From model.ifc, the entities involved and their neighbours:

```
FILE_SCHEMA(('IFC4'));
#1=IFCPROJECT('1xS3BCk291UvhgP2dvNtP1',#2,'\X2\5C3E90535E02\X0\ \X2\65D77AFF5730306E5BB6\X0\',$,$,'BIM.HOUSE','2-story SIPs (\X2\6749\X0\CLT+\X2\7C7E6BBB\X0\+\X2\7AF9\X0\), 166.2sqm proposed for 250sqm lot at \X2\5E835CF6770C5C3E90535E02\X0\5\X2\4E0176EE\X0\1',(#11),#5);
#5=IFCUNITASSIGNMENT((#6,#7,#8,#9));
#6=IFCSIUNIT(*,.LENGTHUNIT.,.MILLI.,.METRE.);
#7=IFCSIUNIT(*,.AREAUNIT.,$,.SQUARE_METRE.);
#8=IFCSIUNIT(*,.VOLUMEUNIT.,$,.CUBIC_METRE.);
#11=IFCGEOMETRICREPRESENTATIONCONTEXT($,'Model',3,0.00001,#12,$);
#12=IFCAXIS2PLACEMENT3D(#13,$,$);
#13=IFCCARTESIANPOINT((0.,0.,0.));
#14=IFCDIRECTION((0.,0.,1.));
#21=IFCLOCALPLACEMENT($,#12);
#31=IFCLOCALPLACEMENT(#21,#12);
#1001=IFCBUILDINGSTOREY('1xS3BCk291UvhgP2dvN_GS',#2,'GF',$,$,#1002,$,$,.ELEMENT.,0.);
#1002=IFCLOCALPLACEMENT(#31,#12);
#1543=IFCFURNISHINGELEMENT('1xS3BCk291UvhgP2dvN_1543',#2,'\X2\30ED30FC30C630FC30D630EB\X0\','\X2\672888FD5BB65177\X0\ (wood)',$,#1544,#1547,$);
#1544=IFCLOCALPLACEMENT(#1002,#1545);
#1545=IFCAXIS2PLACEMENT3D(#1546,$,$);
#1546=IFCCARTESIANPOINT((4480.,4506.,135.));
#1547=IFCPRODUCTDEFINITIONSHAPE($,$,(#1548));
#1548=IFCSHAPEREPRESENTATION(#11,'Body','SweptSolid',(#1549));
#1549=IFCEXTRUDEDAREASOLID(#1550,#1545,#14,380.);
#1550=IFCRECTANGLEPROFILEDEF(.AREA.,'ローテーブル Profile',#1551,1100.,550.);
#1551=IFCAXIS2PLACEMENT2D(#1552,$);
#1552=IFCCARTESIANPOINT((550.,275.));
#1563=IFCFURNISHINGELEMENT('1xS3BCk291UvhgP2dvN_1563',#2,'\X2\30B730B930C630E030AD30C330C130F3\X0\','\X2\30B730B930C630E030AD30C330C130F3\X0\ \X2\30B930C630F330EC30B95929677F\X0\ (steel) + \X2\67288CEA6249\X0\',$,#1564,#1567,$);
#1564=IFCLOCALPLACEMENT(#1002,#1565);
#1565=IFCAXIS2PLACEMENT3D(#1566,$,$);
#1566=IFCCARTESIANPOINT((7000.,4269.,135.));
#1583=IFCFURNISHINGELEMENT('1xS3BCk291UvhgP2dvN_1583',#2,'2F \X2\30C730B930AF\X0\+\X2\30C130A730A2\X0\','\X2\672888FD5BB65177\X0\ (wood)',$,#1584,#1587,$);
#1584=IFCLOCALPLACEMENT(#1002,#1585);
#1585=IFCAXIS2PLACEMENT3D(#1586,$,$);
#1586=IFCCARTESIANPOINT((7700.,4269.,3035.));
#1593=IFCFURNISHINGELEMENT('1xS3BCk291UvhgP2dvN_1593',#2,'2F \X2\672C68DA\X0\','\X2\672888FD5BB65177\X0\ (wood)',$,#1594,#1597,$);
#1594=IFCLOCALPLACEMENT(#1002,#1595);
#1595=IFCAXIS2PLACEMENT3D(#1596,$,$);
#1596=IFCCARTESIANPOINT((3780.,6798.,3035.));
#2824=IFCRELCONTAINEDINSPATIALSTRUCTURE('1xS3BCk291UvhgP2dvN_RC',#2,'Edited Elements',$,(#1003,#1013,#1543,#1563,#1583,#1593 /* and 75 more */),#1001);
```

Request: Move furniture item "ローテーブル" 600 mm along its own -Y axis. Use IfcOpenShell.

```python
import ifcopenshell
import ifcopenshell.api.geometry
import ifcopenshell.util.placement
import ifcopenshell.util.unit

model = ifcopenshell.open("model.ifc")
unit_scale = ifcopenshell.util.unit.calculate_unit_scale(model)

item = model.by_guid("1xS3BCk291UvhgP2dvN_1543")
matrix = ifcopenshell.util.placement.get_local_placement(item.ObjectPlacement)
matrix[:3, 3] -= matrix[:3, 1] * 0.6 / unit_scale
ifcopenshell.api.geometry.edit_object_placement(model, product=item, matrix=matrix, is_si=False)

print(ifcopenshell.util.placement.get_local_placement(item.ObjectPlacement).round(3) + 0.0)

model.write("model-out.ifc")
```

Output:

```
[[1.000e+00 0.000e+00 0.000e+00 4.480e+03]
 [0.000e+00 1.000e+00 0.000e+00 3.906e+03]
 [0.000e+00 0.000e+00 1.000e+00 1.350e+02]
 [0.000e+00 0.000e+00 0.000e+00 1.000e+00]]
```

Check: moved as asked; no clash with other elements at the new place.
